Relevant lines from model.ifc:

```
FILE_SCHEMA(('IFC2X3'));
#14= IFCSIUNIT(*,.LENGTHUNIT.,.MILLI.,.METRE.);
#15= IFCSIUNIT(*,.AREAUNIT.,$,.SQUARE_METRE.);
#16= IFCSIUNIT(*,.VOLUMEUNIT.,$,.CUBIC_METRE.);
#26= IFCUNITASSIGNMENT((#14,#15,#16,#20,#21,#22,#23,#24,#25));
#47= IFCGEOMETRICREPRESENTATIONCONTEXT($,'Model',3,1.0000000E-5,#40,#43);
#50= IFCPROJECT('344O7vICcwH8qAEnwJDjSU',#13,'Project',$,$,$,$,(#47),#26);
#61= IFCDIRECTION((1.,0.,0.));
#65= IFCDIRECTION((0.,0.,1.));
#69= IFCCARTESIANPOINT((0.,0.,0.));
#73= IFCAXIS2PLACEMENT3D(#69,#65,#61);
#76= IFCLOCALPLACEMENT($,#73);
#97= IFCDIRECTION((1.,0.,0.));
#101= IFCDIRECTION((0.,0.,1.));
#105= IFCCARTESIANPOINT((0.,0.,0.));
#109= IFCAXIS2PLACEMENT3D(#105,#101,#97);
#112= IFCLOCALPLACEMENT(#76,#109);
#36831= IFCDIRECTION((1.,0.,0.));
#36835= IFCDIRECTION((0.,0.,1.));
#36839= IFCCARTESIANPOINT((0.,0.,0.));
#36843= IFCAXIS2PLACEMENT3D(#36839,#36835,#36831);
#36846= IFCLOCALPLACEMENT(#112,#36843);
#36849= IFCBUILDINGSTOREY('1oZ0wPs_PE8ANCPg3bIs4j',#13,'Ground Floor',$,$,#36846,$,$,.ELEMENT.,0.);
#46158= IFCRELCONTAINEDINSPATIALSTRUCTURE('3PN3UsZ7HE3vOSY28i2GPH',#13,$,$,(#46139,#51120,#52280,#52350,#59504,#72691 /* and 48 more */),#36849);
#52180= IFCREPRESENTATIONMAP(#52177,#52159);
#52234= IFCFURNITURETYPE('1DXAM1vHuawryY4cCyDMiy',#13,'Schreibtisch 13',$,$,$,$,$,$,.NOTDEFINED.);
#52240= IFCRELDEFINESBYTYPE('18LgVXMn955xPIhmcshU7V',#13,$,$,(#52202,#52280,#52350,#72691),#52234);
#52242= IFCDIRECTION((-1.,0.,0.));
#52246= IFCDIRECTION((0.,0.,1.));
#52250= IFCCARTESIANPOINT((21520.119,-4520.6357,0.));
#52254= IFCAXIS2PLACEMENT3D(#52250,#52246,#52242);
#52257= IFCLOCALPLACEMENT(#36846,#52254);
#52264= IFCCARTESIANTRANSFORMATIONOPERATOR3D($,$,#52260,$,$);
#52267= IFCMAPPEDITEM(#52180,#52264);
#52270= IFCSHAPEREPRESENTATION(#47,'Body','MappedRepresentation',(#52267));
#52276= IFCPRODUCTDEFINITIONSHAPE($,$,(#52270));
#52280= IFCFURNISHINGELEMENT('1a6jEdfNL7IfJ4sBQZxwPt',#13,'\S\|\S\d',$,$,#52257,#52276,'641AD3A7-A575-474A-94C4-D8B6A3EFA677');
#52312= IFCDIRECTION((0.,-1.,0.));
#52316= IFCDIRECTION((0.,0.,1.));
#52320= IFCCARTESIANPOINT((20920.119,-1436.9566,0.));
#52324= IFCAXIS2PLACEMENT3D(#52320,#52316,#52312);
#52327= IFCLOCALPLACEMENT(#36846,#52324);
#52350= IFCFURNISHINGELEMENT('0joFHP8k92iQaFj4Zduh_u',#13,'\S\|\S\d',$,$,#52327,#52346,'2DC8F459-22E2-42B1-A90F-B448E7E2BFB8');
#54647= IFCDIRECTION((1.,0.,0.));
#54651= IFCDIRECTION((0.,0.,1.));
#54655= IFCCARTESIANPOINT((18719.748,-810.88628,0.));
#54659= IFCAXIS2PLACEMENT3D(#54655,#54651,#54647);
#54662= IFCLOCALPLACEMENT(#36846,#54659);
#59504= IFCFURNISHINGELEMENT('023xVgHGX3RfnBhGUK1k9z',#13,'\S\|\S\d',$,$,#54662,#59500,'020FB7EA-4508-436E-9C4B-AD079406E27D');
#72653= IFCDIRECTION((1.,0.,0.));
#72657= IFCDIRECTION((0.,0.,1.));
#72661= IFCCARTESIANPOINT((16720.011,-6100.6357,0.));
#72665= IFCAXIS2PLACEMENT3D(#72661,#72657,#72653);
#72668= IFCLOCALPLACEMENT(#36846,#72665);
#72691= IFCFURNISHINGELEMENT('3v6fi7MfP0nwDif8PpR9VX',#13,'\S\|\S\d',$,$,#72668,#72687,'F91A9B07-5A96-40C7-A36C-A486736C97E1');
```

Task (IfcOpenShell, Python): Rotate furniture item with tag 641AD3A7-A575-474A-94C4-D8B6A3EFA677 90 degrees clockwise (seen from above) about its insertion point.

```python
import ifcopenshell
import ifcopenshell.api.geometry
import ifcopenshell.util.placement

model = ifcopenshell.open("model.ifc")

item = model.by_guid("1a6jEdfNL7IfJ4sBQZxwPt")
matrix = ifcopenshell.util.placement.get_local_placement(item.ObjectPlacement)
matrix = matrix @ ifcopenshell.util.placement.rotation(-90, "Z")
ifcopenshell.api.geometry.edit_object_placement(model, product=item, matrix=matrix, is_si=False)

print(ifcopenshell.util.placement.get_local_placement(item.ObjectPlacement).round(3) + 0.0)

model.write("model_updated.ifc")
```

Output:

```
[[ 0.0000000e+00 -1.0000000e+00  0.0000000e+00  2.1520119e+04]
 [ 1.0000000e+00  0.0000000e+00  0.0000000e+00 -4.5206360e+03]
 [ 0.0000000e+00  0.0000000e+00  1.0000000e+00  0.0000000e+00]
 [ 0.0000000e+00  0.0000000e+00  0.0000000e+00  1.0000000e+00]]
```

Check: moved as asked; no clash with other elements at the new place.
